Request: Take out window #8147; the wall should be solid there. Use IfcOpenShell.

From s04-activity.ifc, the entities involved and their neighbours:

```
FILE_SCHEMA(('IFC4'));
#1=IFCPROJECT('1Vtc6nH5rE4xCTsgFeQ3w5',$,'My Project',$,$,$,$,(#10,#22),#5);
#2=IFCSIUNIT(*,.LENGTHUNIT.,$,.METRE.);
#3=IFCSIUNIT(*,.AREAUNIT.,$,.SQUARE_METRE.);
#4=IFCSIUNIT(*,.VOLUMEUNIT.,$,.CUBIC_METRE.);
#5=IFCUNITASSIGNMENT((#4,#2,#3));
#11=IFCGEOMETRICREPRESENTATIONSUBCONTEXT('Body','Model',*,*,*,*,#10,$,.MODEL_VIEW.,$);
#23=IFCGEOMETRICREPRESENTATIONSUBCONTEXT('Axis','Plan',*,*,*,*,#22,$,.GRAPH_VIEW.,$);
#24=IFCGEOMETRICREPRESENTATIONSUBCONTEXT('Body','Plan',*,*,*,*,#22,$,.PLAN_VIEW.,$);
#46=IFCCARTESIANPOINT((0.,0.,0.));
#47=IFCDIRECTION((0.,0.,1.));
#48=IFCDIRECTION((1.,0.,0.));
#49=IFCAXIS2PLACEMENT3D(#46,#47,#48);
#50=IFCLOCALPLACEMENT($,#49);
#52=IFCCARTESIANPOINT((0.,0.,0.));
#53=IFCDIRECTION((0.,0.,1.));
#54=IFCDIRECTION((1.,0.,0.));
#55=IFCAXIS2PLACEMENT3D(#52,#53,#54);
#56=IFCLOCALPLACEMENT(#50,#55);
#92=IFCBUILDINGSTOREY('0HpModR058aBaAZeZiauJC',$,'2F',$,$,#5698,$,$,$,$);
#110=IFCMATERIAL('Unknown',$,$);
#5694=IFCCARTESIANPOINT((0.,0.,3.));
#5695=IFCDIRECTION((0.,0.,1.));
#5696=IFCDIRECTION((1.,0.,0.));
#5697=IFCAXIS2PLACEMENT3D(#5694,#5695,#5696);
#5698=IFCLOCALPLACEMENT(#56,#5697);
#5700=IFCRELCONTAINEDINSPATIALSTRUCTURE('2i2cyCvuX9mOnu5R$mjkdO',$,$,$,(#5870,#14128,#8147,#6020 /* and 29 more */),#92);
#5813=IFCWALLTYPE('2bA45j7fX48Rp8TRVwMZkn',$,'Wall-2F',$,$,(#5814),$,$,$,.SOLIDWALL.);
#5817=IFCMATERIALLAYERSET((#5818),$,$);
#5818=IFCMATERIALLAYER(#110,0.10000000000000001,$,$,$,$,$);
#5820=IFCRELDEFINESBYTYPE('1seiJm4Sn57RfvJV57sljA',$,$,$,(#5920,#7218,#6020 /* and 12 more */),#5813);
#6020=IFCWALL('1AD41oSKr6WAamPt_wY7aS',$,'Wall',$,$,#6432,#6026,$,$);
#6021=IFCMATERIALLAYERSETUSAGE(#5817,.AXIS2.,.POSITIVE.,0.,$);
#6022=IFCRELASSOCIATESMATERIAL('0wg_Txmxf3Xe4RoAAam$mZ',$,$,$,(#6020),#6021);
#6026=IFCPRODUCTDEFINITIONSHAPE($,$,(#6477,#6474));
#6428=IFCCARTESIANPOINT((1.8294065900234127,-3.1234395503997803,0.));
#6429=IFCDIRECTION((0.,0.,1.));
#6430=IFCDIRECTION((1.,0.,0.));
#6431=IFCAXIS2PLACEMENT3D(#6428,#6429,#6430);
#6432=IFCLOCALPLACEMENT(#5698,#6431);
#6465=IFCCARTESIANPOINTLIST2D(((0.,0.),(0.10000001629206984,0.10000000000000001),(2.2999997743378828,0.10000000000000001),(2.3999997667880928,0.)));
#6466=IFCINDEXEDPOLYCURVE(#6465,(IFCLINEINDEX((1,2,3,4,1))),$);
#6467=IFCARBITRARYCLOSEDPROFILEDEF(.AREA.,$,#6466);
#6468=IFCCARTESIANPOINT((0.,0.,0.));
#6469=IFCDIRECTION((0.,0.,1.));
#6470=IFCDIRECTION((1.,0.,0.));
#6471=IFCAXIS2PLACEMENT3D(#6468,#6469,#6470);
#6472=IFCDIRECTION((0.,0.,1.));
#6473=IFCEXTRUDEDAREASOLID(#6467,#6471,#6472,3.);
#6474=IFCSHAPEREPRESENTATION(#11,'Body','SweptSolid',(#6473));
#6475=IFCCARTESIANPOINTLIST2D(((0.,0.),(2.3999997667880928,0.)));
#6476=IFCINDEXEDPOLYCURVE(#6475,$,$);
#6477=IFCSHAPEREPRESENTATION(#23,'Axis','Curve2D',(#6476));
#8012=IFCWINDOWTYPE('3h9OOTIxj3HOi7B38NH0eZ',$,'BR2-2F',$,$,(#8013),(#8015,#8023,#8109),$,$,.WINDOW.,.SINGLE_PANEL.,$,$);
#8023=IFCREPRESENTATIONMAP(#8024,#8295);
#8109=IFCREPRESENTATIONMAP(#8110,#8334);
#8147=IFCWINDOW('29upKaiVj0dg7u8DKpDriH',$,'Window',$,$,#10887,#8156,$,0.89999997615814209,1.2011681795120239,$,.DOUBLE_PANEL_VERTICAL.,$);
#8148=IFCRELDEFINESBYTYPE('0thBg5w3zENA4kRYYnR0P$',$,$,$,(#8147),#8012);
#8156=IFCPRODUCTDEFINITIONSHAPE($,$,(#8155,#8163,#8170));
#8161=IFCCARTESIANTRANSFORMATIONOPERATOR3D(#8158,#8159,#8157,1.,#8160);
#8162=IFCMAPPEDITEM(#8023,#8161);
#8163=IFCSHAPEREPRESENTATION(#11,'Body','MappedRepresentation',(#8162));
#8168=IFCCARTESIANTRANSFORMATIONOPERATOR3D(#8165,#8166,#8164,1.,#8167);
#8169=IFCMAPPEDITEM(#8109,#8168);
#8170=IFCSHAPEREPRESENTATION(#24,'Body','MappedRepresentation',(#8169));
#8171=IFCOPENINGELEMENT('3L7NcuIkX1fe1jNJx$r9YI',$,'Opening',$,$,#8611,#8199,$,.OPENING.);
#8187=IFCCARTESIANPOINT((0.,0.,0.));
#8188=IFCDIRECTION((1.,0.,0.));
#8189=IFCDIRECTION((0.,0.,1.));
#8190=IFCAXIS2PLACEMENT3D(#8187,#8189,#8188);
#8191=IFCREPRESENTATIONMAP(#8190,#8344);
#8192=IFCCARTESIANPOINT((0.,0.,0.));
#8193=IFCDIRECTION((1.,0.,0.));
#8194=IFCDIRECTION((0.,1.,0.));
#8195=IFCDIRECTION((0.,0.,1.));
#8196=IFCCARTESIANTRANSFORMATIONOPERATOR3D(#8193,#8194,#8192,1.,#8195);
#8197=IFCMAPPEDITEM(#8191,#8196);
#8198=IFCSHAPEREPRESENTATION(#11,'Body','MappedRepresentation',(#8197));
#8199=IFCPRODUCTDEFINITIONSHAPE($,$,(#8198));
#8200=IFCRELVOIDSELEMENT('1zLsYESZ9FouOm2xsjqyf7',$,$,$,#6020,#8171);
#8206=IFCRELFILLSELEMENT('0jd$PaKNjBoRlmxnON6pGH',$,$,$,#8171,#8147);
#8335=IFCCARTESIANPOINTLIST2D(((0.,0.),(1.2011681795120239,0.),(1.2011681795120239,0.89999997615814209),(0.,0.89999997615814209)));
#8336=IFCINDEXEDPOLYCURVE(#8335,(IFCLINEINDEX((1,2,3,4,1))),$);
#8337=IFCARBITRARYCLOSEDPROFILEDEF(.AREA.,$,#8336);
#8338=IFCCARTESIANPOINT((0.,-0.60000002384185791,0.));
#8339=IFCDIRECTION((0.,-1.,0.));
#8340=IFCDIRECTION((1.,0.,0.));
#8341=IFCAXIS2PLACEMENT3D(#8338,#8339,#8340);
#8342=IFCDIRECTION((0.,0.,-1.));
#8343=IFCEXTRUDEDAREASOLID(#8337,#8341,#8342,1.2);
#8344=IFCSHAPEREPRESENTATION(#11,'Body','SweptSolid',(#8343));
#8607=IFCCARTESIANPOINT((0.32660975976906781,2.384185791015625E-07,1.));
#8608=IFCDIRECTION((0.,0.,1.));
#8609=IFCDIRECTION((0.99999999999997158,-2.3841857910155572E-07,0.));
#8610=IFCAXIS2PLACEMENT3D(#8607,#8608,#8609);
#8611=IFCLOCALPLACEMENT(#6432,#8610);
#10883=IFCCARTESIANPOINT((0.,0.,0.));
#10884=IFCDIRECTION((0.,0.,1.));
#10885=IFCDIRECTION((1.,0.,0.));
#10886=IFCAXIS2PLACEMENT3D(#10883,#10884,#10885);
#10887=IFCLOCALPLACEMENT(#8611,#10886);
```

```python
import ifcopenshell
import ifcopenshell.api.feature
import ifcopenshell.api.root
import ifcopenshell.geom
import ifcopenshell.util.shape

model = ifcopenshell.open("s04-activity.ifc")
settings = ifcopenshell.geom.settings()


def volume(element):
    """Net volume in cubic metres, openings subtracted."""
    shape = ifcopenshell.geom.create_shape(settings, element)
    return ifcopenshell.util.shape.get_volume(shape.geometry)


window = model.by_guid("29upKaiVj0dg7u8DKpDriH")
opening = window.FillsVoids[0].RelatingOpeningElement
wall = opening.VoidsElements[0].RelatingBuildingElement
before = volume(wall)

ifcopenshell.api.root.remove_product(model, product=window)
ifcopenshell.api.feature.remove_feature(model, feature=opening)

after = volume(wall)

print(f"wall volume {before:.3f} -> {after:.3f} m3")

model.write("s04-activity_updated.ifc")
```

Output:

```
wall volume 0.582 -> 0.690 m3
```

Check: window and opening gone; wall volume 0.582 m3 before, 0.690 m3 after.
